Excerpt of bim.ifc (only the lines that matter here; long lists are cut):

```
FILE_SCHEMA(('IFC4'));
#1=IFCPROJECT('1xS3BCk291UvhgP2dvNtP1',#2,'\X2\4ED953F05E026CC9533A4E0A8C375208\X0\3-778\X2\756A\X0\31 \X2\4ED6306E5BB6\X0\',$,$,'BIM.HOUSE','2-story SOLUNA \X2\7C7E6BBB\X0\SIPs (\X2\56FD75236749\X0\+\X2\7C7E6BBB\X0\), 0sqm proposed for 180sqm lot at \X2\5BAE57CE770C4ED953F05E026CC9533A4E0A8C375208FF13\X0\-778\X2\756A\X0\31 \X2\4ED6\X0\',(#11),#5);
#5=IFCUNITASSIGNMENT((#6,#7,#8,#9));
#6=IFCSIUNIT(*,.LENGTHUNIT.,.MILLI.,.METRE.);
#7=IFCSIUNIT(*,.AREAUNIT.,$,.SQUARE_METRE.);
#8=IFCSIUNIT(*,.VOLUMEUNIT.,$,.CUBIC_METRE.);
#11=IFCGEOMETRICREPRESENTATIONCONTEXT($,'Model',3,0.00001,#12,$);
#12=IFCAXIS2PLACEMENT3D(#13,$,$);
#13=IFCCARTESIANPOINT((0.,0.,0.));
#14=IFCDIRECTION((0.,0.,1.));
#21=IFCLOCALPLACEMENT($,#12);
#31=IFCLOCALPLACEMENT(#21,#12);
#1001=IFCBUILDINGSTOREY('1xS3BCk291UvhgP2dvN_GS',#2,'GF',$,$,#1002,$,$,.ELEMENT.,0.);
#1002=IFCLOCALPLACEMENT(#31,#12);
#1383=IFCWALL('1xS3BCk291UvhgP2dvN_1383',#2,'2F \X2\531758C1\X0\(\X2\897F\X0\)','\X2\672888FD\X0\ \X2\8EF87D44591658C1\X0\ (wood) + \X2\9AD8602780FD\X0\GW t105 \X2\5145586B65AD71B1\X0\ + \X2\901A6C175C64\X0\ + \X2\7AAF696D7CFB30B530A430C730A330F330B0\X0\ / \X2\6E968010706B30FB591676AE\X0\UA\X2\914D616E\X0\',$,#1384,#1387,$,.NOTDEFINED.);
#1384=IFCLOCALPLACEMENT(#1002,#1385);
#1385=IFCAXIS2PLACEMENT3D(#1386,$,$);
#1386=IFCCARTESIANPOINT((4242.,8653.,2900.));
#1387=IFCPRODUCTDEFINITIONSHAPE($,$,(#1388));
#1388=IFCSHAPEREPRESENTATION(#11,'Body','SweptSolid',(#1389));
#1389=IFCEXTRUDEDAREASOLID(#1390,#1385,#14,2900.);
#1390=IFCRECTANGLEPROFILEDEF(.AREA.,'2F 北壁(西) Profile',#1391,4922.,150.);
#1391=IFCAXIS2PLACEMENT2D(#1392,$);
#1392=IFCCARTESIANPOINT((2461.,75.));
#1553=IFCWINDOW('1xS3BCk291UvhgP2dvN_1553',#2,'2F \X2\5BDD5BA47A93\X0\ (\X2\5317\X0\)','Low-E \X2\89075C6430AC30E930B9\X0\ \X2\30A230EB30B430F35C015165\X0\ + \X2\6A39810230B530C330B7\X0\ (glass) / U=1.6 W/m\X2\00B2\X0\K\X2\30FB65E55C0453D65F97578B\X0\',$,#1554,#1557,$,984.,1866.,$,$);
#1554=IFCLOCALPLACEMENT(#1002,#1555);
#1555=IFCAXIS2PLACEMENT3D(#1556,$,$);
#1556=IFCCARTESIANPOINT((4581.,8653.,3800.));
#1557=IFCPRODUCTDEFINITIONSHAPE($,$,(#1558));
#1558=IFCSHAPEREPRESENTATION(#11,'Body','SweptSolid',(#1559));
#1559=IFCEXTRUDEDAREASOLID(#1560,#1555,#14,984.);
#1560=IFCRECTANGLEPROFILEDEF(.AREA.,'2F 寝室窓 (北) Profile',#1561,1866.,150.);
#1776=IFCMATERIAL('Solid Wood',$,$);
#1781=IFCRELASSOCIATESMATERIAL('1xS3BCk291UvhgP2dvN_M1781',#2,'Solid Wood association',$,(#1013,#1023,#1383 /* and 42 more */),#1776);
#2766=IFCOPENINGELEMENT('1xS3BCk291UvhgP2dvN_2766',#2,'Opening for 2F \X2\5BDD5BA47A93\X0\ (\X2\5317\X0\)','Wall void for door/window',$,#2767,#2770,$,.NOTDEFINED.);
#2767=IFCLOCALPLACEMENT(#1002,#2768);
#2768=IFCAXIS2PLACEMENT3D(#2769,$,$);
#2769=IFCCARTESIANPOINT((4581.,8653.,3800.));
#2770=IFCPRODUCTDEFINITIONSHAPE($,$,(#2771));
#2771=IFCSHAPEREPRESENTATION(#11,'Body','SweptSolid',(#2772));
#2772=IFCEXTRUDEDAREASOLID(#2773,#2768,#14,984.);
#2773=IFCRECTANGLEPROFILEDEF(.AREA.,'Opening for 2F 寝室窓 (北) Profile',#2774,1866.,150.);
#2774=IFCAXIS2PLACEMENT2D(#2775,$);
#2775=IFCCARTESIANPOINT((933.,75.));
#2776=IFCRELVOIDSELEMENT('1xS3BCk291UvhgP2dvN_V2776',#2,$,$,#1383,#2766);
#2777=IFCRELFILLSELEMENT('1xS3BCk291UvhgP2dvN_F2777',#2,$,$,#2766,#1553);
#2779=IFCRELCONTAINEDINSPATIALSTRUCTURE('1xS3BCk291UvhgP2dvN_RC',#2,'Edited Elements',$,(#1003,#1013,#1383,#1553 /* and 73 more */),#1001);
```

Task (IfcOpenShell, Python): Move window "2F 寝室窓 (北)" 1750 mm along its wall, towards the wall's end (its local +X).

```python
import ifcopenshell
import ifcopenshell.api.geometry
import ifcopenshell.util.placement

model = ifcopenshell.open("bim.ifc")

window = model.by_guid("1xS3BCk291UvhgP2dvN_1553")
opening = window.FillsVoids[0].RelatingOpeningElement
wall = opening.VoidsElements[0].RelatingBuildingElement

wall_matrix = ifcopenshell.util.placement.get_local_placement(wall.ObjectPlacement)
shift = wall_matrix[:3, 0] * 1750.0
before = ifcopenshell.util.placement.get_local_placement(window.ObjectPlacement)[:3, 3].copy()

# The window is not placed relative to its opening, so move both.
for product in (opening, window):
    matrix = ifcopenshell.util.placement.get_local_placement(product.ObjectPlacement)
    matrix[:3, 3] += shift
    ifcopenshell.api.geometry.edit_object_placement(model, product=product, matrix=matrix, is_si=False)

after = ifcopenshell.util.placement.get_local_placement(window.ObjectPlacement)[:3, 3]
print("window moved by", (after - before).round(3) + 0.0)

model.write("bim_rev.ifc")
```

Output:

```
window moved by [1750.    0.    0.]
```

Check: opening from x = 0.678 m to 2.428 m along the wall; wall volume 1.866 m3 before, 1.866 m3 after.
